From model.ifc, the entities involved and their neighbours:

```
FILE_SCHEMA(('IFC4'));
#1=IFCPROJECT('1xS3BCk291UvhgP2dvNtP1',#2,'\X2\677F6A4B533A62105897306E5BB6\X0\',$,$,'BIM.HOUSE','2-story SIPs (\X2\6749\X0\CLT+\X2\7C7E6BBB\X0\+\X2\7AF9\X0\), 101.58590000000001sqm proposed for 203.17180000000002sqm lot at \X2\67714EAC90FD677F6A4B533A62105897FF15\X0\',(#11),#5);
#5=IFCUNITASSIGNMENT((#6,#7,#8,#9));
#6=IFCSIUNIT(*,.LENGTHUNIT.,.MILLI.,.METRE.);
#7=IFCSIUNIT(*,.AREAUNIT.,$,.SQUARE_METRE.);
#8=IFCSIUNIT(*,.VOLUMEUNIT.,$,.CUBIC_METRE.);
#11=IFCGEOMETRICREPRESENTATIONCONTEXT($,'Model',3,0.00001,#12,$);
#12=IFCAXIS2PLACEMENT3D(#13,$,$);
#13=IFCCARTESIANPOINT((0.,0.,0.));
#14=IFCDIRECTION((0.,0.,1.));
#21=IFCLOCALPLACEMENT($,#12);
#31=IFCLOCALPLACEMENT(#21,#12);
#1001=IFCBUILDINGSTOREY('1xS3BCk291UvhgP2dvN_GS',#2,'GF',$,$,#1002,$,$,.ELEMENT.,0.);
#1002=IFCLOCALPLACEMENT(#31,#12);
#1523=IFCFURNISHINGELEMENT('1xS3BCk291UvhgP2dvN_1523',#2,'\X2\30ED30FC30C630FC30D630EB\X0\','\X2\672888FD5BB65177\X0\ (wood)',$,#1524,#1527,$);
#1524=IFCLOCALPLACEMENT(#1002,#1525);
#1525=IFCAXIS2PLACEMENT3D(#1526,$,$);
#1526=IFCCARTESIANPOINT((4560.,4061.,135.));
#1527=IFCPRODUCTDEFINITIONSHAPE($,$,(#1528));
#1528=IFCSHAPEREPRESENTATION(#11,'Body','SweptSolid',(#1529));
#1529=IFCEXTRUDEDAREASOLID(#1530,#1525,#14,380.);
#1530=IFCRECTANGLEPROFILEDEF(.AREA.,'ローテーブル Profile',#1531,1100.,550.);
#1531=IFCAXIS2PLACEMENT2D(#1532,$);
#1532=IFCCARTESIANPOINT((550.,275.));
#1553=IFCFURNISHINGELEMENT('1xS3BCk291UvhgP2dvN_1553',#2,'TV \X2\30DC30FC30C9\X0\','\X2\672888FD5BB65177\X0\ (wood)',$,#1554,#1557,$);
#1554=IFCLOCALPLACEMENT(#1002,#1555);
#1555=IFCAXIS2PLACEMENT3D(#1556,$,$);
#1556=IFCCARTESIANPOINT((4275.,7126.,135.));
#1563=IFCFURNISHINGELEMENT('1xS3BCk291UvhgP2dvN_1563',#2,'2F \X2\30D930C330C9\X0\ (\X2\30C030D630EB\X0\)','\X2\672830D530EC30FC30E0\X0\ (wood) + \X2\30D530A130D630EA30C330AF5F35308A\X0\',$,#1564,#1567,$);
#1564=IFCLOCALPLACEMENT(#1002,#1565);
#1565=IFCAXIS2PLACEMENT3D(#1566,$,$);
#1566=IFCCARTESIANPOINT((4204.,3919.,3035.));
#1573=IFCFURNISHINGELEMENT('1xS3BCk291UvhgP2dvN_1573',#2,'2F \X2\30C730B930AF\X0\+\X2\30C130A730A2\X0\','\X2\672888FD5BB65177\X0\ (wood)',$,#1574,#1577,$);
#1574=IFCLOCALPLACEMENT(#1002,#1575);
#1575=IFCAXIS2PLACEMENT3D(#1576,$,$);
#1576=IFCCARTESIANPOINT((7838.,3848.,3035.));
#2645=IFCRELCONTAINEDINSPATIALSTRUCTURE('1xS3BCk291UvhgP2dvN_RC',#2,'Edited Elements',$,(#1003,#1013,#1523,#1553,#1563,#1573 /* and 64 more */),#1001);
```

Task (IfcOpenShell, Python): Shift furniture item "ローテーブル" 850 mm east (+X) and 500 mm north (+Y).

```python
import ifcopenshell
import ifcopenshell.api.geometry
import ifcopenshell.util.placement

model = ifcopenshell.open("model.ifc")

item = model.by_guid("1xS3BCk291UvhgP2dvN_1523")
matrix = ifcopenshell.util.placement.get_local_placement(item.ObjectPlacement)
matrix[0, 3] += 850.0
matrix[1, 3] += 500.0
ifcopenshell.api.geometry.edit_object_placement(model, product=item, matrix=matrix, is_si=False)

print(ifcopenshell.util.placement.get_local_placement(item.ObjectPlacement).round(3) + 0.0)

model.write("model-out.ifc")
```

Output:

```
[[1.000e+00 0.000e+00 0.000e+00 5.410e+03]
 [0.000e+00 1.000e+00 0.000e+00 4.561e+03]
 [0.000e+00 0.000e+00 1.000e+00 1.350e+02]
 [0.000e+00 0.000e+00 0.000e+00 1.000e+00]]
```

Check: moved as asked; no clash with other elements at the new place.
